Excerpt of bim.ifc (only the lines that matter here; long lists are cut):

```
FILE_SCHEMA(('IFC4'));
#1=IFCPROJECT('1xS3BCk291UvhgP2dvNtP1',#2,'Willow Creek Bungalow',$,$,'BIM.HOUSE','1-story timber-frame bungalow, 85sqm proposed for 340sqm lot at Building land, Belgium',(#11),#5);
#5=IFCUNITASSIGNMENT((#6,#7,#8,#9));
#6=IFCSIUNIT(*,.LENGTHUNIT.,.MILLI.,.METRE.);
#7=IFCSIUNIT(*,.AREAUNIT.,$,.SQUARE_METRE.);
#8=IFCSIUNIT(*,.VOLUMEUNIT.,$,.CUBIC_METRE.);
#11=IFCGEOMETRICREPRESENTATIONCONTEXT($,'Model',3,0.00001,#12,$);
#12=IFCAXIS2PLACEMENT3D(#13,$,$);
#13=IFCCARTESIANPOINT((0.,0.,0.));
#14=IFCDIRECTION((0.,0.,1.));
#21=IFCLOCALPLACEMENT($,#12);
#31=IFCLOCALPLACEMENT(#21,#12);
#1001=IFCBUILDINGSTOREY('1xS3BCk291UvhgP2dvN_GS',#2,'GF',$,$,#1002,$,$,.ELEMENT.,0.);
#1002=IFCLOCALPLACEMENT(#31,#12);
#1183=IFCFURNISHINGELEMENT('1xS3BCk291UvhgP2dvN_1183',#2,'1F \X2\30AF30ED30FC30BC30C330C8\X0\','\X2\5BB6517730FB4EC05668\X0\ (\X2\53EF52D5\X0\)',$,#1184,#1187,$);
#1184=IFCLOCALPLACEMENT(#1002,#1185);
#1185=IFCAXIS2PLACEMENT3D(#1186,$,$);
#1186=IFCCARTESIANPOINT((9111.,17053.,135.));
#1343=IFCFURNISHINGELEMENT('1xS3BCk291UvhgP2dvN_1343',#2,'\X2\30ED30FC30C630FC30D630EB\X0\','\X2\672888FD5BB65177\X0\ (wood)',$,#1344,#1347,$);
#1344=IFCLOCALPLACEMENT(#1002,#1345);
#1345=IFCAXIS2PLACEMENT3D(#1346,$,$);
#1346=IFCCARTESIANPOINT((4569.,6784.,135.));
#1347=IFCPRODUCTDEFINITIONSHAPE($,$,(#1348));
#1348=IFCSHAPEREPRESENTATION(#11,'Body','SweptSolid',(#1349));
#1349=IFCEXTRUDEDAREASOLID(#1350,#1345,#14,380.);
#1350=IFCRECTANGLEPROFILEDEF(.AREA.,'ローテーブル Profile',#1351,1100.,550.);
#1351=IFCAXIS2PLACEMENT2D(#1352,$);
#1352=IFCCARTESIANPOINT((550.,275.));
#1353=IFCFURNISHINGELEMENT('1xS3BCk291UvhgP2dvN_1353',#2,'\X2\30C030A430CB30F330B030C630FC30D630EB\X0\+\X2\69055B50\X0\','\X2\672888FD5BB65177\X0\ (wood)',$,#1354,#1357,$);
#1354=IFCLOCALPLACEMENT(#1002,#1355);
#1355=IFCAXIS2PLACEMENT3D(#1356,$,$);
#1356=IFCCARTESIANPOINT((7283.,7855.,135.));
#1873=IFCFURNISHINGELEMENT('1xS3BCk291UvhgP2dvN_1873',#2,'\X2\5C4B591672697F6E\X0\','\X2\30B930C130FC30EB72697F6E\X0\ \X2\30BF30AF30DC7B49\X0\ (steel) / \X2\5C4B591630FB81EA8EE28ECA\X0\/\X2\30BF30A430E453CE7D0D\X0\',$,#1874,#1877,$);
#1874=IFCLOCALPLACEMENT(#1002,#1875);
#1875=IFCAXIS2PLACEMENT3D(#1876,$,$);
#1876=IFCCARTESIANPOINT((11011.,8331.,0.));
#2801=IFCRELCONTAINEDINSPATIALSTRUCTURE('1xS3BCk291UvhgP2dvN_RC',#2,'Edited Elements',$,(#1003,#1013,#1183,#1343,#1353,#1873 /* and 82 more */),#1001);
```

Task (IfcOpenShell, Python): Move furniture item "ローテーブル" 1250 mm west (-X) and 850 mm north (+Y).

```python
import ifcopenshell
import ifcopenshell.api.geometry
import ifcopenshell.util.placement
import ifcopenshell.util.unit

model = ifcopenshell.open("bim.ifc")
unit_scale = ifcopenshell.util.unit.calculate_unit_scale(model)

item = model.by_guid("1xS3BCk291UvhgP2dvN_1343")
matrix = ifcopenshell.util.placement.get_local_placement(item.ObjectPlacement)
matrix[0, 3] -= 1.25 / unit_scale
matrix[1, 3] += 0.85 / unit_scale
ifcopenshell.api.geometry.edit_object_placement(model, product=item, matrix=matrix, is_si=False)

print(ifcopenshell.util.placement.get_local_placement(item.ObjectPlacement).round(3) + 0.0)

model.write("bim_updated.ifc")
```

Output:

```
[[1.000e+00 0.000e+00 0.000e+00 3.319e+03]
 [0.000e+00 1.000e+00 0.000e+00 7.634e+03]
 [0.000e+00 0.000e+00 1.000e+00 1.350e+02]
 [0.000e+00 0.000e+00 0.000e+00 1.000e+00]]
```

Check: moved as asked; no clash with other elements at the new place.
